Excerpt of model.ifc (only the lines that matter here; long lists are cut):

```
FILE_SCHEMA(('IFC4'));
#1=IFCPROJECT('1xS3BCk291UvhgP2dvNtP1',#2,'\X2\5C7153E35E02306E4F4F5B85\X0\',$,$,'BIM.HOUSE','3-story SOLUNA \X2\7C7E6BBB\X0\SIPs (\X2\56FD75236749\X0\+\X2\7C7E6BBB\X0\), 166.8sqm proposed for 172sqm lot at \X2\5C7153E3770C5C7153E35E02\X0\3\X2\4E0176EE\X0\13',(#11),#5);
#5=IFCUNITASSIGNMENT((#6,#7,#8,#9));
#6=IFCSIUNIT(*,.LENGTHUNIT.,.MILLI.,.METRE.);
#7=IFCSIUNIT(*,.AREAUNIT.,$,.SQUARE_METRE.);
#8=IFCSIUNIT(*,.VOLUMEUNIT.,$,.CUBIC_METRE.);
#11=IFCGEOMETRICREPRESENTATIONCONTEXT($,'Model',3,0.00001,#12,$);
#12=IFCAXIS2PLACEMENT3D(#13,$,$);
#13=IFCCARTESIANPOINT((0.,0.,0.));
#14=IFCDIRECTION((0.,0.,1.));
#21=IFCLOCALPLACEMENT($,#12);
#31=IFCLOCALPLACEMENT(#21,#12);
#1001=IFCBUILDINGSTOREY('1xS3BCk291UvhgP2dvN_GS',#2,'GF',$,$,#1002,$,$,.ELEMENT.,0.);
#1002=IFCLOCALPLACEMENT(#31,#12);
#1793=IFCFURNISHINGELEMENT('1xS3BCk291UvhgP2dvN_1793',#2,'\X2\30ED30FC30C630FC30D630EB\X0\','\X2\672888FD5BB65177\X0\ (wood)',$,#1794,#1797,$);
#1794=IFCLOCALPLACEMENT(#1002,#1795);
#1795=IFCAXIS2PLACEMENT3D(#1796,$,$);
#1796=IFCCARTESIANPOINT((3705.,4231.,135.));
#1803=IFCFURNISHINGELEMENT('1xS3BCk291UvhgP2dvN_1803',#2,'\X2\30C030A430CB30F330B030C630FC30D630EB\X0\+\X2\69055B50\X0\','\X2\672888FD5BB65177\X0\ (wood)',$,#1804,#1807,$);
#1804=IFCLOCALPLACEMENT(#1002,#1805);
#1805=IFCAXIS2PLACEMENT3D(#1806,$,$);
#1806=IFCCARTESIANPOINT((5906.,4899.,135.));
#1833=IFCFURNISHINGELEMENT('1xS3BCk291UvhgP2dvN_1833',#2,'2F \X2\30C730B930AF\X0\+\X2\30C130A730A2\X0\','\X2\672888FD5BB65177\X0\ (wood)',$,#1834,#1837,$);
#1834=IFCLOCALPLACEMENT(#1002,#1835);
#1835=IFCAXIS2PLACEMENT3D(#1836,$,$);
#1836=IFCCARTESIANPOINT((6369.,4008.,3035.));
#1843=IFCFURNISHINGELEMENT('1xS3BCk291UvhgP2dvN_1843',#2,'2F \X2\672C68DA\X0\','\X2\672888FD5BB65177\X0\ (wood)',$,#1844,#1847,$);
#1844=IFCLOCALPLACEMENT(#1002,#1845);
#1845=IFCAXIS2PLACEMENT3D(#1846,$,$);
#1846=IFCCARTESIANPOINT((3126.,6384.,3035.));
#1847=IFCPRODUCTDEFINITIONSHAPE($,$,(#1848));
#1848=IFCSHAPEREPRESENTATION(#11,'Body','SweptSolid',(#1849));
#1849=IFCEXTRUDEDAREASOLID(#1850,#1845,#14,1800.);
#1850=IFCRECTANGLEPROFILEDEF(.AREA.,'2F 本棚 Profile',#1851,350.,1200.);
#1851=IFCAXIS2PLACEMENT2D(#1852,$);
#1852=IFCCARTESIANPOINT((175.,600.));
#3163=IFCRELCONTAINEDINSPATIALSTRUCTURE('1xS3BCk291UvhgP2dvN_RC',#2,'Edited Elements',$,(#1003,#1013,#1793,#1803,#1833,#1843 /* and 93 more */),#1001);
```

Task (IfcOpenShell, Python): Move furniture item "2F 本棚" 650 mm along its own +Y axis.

```python
import ifcopenshell
import ifcopenshell.api.geometry
import ifcopenshell.util.placement

model = ifcopenshell.open("model.ifc")

item = model.by_id(1843)
matrix = ifcopenshell.util.placement.get_local_placement(item.ObjectPlacement)
matrix[:3, 3] += matrix[:3, 1] * 650.0
ifcopenshell.api.geometry.edit_object_placement(model, product=item, matrix=matrix, is_si=False)

print(ifcopenshell.util.placement.get_local_placement(item.ObjectPlacement).round(3) + 0.0)

model.write("model_v2.ifc")
```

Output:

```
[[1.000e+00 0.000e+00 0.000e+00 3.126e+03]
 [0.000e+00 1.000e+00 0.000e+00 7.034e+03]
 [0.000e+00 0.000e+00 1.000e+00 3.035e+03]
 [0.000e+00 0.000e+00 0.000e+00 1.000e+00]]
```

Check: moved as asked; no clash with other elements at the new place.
